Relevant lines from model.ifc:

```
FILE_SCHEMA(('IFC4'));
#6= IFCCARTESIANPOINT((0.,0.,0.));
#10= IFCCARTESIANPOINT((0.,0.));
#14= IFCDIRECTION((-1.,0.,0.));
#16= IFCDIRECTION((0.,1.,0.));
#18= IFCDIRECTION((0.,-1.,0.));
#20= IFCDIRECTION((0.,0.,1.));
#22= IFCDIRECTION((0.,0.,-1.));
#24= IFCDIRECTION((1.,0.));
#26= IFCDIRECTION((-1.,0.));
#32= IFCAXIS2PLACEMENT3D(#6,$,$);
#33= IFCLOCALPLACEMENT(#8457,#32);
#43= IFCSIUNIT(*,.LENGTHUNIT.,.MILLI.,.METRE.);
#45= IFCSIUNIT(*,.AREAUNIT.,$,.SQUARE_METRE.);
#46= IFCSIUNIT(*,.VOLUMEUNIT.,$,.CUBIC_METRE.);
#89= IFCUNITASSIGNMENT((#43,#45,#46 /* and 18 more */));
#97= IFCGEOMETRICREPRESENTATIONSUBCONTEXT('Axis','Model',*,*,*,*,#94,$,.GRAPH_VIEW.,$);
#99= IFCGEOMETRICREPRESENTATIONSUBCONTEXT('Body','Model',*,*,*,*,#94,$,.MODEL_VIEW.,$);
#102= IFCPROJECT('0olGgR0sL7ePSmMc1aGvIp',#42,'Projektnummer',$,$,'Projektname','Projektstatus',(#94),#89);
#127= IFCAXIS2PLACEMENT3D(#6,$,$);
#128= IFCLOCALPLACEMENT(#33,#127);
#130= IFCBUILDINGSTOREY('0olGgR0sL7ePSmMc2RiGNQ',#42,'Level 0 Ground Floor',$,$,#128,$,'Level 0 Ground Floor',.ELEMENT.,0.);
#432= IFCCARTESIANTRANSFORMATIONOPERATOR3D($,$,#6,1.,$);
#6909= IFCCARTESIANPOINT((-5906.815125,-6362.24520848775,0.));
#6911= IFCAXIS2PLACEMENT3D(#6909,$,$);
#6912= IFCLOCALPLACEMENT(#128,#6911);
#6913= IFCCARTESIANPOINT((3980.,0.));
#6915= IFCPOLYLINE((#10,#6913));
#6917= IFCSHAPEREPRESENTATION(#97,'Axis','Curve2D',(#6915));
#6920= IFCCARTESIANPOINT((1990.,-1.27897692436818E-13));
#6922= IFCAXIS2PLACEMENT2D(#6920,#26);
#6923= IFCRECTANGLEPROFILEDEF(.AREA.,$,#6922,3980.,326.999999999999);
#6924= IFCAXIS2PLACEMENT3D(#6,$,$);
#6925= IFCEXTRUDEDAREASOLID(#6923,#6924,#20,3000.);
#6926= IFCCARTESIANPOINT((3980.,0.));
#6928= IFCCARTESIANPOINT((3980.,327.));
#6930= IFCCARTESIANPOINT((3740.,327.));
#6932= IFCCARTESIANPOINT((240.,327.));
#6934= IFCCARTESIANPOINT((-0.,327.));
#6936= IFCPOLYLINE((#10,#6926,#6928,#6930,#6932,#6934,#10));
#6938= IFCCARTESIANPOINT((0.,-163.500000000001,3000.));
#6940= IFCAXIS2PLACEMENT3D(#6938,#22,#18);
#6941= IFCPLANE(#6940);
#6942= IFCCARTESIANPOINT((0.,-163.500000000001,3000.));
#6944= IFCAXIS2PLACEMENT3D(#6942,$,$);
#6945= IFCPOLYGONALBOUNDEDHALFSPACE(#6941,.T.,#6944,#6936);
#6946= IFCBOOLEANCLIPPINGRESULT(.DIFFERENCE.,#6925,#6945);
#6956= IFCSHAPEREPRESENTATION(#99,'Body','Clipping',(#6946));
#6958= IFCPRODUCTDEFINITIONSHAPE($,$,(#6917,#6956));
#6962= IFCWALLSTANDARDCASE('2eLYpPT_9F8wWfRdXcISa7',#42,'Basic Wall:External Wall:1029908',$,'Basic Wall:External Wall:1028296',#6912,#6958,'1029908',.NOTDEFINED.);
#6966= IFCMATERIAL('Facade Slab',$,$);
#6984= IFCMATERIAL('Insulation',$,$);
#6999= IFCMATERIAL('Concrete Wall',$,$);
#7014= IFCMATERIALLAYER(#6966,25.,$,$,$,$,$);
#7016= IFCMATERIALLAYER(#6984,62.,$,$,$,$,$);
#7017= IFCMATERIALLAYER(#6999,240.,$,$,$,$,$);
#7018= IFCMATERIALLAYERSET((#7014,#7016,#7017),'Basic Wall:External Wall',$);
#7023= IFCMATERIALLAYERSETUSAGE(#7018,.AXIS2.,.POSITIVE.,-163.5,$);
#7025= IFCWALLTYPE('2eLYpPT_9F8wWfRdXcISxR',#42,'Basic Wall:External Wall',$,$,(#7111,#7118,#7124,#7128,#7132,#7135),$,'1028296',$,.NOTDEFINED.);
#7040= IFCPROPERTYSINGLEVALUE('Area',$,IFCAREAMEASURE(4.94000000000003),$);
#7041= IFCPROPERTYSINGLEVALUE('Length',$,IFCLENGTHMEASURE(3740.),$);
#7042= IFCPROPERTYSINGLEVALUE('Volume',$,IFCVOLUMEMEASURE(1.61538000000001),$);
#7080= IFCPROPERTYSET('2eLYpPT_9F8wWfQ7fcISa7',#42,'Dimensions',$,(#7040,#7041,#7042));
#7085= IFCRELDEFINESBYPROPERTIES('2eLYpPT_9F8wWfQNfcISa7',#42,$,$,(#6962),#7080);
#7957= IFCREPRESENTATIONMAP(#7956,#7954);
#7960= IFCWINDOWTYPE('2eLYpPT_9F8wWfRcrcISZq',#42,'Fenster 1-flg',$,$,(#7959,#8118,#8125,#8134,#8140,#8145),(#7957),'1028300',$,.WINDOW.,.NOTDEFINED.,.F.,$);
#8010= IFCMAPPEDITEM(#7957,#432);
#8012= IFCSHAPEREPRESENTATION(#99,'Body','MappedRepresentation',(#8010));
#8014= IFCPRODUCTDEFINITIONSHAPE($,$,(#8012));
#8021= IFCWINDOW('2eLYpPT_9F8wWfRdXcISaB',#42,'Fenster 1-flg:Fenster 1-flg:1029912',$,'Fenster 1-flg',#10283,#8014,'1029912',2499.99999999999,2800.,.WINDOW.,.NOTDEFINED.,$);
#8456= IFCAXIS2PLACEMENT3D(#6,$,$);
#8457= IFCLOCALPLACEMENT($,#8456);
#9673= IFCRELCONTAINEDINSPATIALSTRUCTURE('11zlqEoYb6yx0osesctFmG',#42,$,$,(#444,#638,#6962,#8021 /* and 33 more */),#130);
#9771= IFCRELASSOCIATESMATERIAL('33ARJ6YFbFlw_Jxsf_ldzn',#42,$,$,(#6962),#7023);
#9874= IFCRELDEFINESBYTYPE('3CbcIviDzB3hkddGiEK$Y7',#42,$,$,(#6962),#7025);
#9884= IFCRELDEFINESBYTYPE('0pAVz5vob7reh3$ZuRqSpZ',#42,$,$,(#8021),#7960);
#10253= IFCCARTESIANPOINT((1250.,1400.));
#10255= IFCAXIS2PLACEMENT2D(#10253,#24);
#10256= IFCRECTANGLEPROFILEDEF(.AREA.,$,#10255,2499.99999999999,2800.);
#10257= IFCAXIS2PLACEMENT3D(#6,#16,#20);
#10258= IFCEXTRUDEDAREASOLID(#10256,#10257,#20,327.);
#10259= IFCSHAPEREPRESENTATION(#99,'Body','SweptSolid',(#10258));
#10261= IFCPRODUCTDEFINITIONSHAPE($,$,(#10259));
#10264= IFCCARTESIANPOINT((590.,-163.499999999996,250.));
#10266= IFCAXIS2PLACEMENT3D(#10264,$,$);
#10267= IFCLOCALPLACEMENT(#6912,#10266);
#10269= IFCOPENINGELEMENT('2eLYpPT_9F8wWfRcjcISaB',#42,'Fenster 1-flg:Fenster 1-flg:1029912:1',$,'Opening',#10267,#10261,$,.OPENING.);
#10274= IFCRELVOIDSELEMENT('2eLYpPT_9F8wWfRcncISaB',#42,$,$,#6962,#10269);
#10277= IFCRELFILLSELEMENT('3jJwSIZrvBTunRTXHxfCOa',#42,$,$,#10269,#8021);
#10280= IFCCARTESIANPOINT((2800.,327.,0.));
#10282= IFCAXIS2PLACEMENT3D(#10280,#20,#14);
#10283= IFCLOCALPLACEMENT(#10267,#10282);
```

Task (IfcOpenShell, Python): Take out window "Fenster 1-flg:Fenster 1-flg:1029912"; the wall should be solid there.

```python
import ifcopenshell
import ifcopenshell.api.feature
import ifcopenshell.api.pset
import ifcopenshell.api.root
import ifcopenshell.geom
import ifcopenshell.util.element
import ifcopenshell.util.shape
import ifcopenshell.util.unit

model = ifcopenshell.open("model.ifc")
area_scale = ifcopenshell.util.unit.calculate_unit_scale(model, "AREAUNIT")
volume_scale = ifcopenshell.util.unit.calculate_unit_scale(model, "VOLUMEUNIT")
settings = ifcopenshell.geom.settings()


def volume(element):
    """Net volume in cubic metres, openings subtracted."""
    shape = ifcopenshell.geom.create_shape(settings, element)
    return ifcopenshell.util.shape.get_volume(shape.geometry)


window = model.by_guid("2eLYpPT_9F8wWfRdXcISaB")
opening = window.FillsVoids[0].RelatingOpeningElement
wall = opening.VoidsElements[0].RelatingBuildingElement
before = volume(wall)

ifcopenshell.api.root.remove_product(model, product=window)
ifcopenshell.api.feature.remove_feature(model, feature=opening)

after = volume(wall)
thickness = 0.327  # wall thickness in metres

# Update the wall's stored quantities.
pset = model.by_id(ifcopenshell.util.element.get_pset(wall, "Dimensions", should_inherit=False)["id"])
ifcopenshell.api.pset.edit_pset(model, pset=pset, properties={
    "Area": model.create_entity("IfcAreaMeasure", after / thickness / area_scale),
    "Volume": model.create_entity("IfcVolumeMeasure", after / volume_scale),
})

print(f"wall volume {before:.3f} -> {after:.3f} m3")

model.write("model_edited.ifc")
```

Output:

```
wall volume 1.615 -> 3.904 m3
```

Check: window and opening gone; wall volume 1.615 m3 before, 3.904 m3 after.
